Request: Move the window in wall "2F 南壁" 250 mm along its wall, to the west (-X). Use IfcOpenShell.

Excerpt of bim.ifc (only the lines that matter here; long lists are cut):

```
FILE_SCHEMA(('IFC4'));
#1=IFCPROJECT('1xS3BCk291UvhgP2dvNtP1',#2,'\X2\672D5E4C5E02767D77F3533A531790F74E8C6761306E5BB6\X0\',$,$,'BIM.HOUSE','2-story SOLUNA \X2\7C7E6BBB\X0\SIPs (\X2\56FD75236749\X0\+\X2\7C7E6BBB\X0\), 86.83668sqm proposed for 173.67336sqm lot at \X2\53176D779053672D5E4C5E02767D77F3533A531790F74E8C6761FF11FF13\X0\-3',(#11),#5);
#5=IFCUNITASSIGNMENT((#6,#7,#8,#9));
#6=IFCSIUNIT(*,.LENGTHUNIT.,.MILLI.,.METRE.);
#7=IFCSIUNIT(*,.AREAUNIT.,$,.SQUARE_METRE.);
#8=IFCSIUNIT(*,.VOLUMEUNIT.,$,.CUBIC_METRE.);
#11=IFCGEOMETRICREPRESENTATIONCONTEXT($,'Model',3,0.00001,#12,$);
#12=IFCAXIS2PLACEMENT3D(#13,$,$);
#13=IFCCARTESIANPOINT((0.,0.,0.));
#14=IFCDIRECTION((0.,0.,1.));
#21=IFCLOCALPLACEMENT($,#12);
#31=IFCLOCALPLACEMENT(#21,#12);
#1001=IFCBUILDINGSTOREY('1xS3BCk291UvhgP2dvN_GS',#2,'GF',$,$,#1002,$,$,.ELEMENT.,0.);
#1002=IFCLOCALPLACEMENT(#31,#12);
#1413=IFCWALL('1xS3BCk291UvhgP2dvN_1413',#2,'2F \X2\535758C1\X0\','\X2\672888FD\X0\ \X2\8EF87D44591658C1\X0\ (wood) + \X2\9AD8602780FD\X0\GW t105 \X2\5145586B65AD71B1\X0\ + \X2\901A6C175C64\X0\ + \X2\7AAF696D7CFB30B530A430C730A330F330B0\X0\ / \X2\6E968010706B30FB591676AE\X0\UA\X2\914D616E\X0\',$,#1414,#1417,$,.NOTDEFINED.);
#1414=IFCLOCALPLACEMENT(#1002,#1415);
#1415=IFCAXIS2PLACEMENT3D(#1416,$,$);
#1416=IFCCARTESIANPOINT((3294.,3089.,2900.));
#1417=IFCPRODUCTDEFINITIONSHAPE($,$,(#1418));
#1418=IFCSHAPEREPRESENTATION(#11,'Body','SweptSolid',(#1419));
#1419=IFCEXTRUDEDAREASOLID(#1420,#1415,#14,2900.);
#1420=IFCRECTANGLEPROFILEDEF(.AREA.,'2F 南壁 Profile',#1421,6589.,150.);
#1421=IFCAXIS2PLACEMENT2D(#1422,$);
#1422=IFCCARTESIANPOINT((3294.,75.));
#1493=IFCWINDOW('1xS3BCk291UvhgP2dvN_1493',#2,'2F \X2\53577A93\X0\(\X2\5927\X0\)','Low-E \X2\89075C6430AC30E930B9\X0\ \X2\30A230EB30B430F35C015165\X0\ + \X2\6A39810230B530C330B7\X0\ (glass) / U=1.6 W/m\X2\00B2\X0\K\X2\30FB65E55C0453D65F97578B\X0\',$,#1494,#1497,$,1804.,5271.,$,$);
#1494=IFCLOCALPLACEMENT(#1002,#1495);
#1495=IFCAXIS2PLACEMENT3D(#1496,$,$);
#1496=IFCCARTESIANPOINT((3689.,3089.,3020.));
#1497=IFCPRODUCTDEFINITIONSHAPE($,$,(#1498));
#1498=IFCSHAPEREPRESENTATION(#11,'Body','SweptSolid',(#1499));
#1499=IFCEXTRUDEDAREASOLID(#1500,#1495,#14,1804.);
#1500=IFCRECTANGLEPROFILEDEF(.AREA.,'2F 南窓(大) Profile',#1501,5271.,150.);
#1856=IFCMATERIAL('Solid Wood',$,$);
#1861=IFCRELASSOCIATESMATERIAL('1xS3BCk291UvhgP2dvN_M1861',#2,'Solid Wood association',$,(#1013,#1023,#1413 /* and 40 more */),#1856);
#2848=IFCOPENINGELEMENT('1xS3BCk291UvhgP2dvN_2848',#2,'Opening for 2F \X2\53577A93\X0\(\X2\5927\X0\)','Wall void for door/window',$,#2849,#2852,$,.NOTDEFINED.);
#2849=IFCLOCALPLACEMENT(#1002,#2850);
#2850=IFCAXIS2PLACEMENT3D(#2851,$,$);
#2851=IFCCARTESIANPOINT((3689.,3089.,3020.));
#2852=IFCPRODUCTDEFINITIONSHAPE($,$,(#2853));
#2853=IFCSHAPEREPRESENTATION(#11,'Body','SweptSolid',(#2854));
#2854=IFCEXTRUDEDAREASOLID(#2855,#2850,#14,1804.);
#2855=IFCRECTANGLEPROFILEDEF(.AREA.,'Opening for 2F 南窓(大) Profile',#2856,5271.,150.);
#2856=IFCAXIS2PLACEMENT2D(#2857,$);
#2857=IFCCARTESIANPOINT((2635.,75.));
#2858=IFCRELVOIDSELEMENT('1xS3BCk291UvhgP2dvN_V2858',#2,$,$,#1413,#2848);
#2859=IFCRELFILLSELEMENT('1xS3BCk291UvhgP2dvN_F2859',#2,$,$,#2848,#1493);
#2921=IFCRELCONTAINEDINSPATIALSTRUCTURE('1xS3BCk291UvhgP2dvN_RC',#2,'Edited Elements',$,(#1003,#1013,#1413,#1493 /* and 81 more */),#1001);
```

```python
import ifcopenshell
import ifcopenshell.api.geometry
import ifcopenshell.util.placement
import ifcopenshell.util.unit

model = ifcopenshell.open("bim.ifc")
unit_scale = ifcopenshell.util.unit.calculate_unit_scale(model)

window = model.by_guid("1xS3BCk291UvhgP2dvN_1493")
opening = window.FillsVoids[0].RelatingOpeningElement
wall = opening.VoidsElements[0].RelatingBuildingElement

wall_matrix = ifcopenshell.util.placement.get_local_placement(wall.ObjectPlacement)
shift = wall_matrix[:3, 0] * -0.25 / unit_scale
before = ifcopenshell.util.placement.get_local_placement(window.ObjectPlacement)[:3, 3].copy()

# The window is not placed relative to its opening, so move both.
for product in (opening, window):
    matrix = ifcopenshell.util.placement.get_local_placement(product.ObjectPlacement)
    matrix[:3, 3] += shift
    ifcopenshell.api.geometry.edit_object_placement(model, product=product, matrix=matrix, is_si=False)

after = ifcopenshell.util.placement.get_local_placement(window.ObjectPlacement)[:3, 3]
print("window moved by", (after - before).round(3) + 0.0)

model.write("bim_updated.ifc")
```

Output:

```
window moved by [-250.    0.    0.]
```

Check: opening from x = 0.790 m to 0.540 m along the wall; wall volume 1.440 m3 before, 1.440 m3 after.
